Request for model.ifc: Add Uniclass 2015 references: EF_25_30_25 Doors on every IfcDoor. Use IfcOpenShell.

First a look at what the model holds.

```python
import ifcopenshell

model = ifcopenshell.open("model.ifc")
print(model.schema)
print("classifications:", [c.Name for c in model.by_type("IfcClassification")])
for ifc_class in ("IfcDoor", "IfcRoof", "IfcStair", "IfcWall", "IfcWindow"):
    print(ifc_class, len(model.by_type(ifc_class)))
```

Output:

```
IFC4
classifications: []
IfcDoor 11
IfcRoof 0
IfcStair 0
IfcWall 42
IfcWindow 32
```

```python
import ifcopenshell
import ifcopenshell.api.classification

model = ifcopenshell.open("model.ifc")

system = ifcopenshell.api.classification.add_classification(model, classification="Uniclass 2015")

codes = {
    "IfcDoor": ("EF_25_30_25", "Doors"),
}
for ifc_class, (code, name) in codes.items():
    products = model.by_type(ifc_class)
    ifcopenshell.api.classification.add_reference(
        model, products=products, classification=system, identification=code, name=name
    )
    print(code, len(products))

model.write("model_rev.ifc")
```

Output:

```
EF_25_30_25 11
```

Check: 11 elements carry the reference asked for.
